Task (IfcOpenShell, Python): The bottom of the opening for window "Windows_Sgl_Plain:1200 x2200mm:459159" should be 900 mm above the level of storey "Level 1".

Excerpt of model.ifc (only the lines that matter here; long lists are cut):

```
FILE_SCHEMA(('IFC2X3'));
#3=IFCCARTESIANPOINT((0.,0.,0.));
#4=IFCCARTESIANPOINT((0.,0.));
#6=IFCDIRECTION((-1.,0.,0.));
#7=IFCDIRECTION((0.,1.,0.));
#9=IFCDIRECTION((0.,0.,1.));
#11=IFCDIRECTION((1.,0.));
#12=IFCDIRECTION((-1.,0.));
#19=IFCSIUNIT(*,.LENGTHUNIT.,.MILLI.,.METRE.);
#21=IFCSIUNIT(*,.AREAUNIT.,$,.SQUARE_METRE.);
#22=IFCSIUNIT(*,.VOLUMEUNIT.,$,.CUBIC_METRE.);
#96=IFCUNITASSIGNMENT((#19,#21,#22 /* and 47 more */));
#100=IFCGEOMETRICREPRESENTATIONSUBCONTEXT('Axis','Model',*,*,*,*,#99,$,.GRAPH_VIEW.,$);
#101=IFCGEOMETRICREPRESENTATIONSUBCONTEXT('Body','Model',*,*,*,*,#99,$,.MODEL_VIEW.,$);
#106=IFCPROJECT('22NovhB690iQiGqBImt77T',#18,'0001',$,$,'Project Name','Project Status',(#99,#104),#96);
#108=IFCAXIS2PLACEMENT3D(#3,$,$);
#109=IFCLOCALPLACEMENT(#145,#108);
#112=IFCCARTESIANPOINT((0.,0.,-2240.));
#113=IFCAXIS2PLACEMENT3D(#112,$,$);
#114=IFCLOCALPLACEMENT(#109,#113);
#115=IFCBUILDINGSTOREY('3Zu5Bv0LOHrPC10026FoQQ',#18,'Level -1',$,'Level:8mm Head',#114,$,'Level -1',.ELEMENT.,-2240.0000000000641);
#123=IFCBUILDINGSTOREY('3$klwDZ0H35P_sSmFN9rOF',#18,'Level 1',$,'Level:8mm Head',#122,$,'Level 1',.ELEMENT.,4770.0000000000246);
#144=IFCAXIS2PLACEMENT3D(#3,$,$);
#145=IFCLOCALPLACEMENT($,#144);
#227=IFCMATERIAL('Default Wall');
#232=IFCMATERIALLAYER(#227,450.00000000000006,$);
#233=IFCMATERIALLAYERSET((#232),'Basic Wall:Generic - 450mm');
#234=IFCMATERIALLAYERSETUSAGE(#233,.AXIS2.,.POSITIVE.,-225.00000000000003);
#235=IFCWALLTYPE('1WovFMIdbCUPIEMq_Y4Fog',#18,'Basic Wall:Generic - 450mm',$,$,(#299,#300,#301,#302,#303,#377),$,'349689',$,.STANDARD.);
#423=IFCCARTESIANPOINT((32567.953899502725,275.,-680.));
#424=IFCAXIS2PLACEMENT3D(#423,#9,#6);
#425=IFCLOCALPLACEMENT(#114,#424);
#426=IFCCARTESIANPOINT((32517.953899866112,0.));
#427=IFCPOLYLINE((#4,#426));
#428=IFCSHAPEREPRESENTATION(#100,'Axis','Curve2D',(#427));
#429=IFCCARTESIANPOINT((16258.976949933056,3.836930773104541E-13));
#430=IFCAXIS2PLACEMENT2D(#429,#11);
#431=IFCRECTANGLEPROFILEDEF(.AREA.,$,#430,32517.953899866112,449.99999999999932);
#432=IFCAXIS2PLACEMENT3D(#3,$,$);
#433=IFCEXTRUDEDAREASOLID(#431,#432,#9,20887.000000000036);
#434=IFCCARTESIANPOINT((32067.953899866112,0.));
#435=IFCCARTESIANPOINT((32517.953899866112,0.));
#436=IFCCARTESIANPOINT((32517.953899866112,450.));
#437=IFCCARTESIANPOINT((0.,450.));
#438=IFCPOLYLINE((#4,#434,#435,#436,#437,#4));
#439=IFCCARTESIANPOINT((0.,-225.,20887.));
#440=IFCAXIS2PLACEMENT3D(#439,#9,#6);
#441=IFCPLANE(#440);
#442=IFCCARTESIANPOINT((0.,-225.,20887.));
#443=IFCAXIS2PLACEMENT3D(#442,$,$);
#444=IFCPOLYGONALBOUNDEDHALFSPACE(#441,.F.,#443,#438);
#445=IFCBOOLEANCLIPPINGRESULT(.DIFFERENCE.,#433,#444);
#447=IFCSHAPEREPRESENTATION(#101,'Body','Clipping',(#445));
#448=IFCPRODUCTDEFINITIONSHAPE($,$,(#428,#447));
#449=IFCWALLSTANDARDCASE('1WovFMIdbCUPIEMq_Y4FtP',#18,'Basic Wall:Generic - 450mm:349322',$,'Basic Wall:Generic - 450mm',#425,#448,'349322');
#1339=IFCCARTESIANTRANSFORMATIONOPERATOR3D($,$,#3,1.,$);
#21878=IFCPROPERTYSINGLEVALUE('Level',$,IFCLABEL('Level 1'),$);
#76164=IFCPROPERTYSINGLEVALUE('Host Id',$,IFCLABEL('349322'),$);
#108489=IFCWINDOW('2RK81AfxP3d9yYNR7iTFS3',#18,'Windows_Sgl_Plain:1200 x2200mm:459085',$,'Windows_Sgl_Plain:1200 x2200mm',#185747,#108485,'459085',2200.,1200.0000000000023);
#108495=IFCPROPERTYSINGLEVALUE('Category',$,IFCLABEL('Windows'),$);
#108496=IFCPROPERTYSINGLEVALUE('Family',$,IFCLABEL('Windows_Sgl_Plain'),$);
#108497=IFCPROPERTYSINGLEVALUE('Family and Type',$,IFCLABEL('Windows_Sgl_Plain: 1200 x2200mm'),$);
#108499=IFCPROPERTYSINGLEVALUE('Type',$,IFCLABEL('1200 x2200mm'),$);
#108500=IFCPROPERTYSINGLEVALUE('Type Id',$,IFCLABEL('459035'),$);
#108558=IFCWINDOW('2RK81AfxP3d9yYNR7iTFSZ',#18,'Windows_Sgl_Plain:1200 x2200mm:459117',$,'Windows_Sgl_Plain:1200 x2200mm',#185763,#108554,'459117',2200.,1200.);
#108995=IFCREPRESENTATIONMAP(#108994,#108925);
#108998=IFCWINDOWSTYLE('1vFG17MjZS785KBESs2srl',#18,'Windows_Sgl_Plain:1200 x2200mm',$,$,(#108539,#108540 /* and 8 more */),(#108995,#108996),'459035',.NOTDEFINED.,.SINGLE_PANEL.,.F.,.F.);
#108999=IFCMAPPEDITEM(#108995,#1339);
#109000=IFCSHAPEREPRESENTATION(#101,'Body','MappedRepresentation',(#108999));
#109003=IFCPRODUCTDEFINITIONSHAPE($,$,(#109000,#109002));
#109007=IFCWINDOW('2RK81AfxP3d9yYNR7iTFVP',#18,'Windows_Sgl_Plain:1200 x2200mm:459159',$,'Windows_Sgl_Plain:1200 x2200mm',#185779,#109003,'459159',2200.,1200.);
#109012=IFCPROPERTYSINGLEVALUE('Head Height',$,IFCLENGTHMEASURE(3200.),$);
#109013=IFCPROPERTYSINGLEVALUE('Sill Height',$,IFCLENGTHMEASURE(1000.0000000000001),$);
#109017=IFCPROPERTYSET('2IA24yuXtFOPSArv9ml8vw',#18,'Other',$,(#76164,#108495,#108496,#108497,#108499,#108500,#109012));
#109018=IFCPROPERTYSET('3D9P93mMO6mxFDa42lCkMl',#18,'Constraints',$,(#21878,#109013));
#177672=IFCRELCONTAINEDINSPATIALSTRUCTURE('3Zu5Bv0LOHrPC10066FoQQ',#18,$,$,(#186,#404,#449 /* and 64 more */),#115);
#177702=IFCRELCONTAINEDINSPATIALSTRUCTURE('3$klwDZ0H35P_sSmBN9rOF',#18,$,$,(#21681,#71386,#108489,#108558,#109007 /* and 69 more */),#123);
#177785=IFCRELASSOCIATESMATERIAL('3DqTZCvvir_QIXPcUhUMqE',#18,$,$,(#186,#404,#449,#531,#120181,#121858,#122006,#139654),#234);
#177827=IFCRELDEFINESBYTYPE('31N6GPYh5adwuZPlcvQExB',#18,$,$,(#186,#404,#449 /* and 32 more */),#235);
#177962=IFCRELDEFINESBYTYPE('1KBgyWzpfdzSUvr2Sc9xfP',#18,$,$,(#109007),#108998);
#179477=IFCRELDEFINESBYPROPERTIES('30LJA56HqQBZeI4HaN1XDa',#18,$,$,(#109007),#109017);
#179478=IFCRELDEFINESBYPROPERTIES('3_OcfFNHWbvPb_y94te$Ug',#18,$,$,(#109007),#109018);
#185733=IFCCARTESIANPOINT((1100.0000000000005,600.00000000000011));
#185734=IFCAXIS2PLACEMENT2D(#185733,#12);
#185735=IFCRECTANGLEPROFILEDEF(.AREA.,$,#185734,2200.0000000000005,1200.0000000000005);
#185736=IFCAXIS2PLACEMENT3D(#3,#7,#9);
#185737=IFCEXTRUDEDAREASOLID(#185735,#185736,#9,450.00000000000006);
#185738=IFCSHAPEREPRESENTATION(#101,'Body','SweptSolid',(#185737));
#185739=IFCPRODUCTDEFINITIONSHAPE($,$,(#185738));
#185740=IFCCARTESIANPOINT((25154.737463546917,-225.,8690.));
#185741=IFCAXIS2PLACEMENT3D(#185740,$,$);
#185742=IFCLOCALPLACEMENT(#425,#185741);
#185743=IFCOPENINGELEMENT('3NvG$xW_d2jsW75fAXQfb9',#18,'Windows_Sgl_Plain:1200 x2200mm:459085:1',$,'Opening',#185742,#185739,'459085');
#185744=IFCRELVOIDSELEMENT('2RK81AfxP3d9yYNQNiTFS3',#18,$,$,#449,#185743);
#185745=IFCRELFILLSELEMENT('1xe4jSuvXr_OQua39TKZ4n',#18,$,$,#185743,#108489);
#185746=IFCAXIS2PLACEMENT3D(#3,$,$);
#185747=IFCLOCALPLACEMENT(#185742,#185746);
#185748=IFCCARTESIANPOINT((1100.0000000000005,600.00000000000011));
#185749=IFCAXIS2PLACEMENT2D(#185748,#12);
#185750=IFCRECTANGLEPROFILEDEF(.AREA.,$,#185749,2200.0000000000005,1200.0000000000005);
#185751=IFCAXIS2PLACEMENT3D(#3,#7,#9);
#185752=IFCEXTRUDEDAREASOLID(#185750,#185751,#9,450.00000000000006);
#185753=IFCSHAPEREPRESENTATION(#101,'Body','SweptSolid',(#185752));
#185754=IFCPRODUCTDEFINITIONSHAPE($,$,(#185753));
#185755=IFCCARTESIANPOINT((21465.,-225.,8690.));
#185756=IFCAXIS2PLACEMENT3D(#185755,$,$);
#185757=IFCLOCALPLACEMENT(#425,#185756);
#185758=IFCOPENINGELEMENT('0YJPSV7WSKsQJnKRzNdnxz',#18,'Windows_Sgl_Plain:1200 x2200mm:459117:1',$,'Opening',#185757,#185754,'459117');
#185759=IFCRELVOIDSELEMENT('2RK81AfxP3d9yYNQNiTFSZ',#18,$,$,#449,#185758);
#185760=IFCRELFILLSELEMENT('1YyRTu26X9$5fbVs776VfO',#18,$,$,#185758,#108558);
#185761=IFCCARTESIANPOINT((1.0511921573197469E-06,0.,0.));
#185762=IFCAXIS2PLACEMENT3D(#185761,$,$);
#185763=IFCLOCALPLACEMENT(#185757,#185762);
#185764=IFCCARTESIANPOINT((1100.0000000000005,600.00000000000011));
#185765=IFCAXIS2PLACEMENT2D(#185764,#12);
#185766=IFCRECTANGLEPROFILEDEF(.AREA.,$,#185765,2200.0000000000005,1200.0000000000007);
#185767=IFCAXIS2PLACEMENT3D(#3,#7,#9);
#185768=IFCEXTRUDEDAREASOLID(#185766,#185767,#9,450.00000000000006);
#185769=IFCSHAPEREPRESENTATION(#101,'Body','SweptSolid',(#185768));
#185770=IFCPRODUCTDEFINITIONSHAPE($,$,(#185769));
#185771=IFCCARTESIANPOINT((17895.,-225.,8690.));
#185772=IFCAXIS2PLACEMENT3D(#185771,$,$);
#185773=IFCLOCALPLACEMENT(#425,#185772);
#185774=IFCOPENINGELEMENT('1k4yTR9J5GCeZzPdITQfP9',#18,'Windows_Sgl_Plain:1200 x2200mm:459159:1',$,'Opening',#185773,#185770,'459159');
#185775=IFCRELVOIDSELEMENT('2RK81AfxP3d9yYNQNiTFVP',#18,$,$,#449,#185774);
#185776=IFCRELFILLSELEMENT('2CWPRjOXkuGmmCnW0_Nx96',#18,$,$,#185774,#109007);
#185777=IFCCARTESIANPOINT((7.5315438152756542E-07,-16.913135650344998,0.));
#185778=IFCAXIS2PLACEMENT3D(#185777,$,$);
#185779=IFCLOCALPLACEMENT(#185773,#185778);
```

```python
import numpy as np
import ifcopenshell
import ifcopenshell.api.geometry
import ifcopenshell.api.pset
import ifcopenshell.geom
import ifcopenshell.util.element
import ifcopenshell.util.placement
import ifcopenshell.util.shape
import ifcopenshell.util.unit

model = ifcopenshell.open("model.ifc")
unit_scale = ifcopenshell.util.unit.calculate_unit_scale(model)

window = model.by_guid("2RK81AfxP3d9yYNR7iTFVP")
opening = window.FillsVoids[0].RelatingOpeningElement
storey = ifcopenshell.util.element.get_container(window, ifc_class="IfcBuildingStorey")
level = ifcopenshell.util.placement.get_local_placement(storey.ObjectPlacement)[2, 3]

# The opening's origin need not be at the sill, so measure its lowest point.
shape = ifcopenshell.geom.create_shape(ifcopenshell.geom.settings(), opening)
bottom = ifcopenshell.util.shape.get_shape_bottom_elevation(shape, shape.geometry) / unit_scale
dz = level + 0.9 / unit_scale - bottom

shift = np.array([0.0, 0.0, dz])
# The window is placed relative to its opening, so it follows when the opening moves.
matrix = ifcopenshell.util.placement.get_local_placement(opening.ObjectPlacement)
matrix[:3, 3] += shift
ifcopenshell.api.geometry.edit_object_placement(
    model, product=opening, matrix=matrix, is_si=False, should_transform_children=True
)

# Keep the stored heights in step.
pset = model.by_id(ifcopenshell.util.element.get_pset(window, "Other", should_inherit=False)["id"])
ifcopenshell.api.pset.edit_pset(model, pset=pset, properties={
    "Head Height": model.create_entity("IfcLengthMeasure", ifcopenshell.util.element.get_pset(window, "Other", "Head Height") + dz),
})
pset = model.by_id(ifcopenshell.util.element.get_pset(window, "Constraints", should_inherit=False)["id"])
ifcopenshell.api.pset.edit_pset(model, pset=pset, properties={
    "Sill Height": model.create_entity("IfcLengthMeasure", ifcopenshell.util.element.get_pset(window, "Constraints", "Sill Height") + dz),
})

print(f"moved by {dz * unit_scale:+.3f} m")

model.write("model_updated.ifc")
```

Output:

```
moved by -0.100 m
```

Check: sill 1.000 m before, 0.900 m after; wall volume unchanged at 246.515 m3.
